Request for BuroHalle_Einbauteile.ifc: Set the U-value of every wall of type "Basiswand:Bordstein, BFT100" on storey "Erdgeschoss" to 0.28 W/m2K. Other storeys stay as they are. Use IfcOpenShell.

First a look at what the model holds.

```python
import ifcopenshell
import ifcopenshell.util.element

model = ifcopenshell.open("BuroHalle_Einbauteile.ifc")
print(model.schema)
storey = next(s for s in model.by_type("IfcBuildingStorey") if s.Name == "Erdgeschoss")
walls = [e for e in ifcopenshell.util.element.get_decomposition(storey) if e.is_a("IfcWall")]
seen = {}
for e in walls:
    element_type = ifcopenshell.util.element.get_type(e)
    key = (element_type.Name if element_type != e and element_type else None, ifcopenshell.util.element.get_pset(e, "Pset_WallCommon", "ThermalTransmittance"))
    seen[key] = seen.get(key, 0) + 1
for (name, value), count in sorted(seen.items(), key=str):
    print(count, "x", name, "|", value)
```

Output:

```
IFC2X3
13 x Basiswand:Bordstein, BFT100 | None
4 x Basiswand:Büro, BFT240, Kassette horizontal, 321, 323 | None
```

```python
import ifcopenshell
import ifcopenshell.api.pset
import ifcopenshell.util.element

model = ifcopenshell.open("BuroHalle_Einbauteile.ifc")

storey = next(s for s in model.by_type("IfcBuildingStorey") if s.Name == "Erdgeschoss")
walls = [e for e in ifcopenshell.util.element.get_decomposition(storey) if e.is_a("IfcWall")]

count = 0
for e in walls:
    element_type = ifcopenshell.util.element.get_type(e)
    if element_type in (None, e) or element_type.Name != "Basiswand:Bordstein, BFT100":
        continue
    # add_pset returns the element's existing set when there is one.
    pset = ifcopenshell.api.pset.add_pset(model, product=e, name="Pset_WallCommon")
    ifcopenshell.api.pset.edit_pset(model, pset=pset, properties={"ThermalTransmittance": 0.28})
    count += 1

print(count, "walls updated")

model.write("BuroHalle_Einbauteile_rev.ifc")
```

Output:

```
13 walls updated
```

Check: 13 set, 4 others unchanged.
